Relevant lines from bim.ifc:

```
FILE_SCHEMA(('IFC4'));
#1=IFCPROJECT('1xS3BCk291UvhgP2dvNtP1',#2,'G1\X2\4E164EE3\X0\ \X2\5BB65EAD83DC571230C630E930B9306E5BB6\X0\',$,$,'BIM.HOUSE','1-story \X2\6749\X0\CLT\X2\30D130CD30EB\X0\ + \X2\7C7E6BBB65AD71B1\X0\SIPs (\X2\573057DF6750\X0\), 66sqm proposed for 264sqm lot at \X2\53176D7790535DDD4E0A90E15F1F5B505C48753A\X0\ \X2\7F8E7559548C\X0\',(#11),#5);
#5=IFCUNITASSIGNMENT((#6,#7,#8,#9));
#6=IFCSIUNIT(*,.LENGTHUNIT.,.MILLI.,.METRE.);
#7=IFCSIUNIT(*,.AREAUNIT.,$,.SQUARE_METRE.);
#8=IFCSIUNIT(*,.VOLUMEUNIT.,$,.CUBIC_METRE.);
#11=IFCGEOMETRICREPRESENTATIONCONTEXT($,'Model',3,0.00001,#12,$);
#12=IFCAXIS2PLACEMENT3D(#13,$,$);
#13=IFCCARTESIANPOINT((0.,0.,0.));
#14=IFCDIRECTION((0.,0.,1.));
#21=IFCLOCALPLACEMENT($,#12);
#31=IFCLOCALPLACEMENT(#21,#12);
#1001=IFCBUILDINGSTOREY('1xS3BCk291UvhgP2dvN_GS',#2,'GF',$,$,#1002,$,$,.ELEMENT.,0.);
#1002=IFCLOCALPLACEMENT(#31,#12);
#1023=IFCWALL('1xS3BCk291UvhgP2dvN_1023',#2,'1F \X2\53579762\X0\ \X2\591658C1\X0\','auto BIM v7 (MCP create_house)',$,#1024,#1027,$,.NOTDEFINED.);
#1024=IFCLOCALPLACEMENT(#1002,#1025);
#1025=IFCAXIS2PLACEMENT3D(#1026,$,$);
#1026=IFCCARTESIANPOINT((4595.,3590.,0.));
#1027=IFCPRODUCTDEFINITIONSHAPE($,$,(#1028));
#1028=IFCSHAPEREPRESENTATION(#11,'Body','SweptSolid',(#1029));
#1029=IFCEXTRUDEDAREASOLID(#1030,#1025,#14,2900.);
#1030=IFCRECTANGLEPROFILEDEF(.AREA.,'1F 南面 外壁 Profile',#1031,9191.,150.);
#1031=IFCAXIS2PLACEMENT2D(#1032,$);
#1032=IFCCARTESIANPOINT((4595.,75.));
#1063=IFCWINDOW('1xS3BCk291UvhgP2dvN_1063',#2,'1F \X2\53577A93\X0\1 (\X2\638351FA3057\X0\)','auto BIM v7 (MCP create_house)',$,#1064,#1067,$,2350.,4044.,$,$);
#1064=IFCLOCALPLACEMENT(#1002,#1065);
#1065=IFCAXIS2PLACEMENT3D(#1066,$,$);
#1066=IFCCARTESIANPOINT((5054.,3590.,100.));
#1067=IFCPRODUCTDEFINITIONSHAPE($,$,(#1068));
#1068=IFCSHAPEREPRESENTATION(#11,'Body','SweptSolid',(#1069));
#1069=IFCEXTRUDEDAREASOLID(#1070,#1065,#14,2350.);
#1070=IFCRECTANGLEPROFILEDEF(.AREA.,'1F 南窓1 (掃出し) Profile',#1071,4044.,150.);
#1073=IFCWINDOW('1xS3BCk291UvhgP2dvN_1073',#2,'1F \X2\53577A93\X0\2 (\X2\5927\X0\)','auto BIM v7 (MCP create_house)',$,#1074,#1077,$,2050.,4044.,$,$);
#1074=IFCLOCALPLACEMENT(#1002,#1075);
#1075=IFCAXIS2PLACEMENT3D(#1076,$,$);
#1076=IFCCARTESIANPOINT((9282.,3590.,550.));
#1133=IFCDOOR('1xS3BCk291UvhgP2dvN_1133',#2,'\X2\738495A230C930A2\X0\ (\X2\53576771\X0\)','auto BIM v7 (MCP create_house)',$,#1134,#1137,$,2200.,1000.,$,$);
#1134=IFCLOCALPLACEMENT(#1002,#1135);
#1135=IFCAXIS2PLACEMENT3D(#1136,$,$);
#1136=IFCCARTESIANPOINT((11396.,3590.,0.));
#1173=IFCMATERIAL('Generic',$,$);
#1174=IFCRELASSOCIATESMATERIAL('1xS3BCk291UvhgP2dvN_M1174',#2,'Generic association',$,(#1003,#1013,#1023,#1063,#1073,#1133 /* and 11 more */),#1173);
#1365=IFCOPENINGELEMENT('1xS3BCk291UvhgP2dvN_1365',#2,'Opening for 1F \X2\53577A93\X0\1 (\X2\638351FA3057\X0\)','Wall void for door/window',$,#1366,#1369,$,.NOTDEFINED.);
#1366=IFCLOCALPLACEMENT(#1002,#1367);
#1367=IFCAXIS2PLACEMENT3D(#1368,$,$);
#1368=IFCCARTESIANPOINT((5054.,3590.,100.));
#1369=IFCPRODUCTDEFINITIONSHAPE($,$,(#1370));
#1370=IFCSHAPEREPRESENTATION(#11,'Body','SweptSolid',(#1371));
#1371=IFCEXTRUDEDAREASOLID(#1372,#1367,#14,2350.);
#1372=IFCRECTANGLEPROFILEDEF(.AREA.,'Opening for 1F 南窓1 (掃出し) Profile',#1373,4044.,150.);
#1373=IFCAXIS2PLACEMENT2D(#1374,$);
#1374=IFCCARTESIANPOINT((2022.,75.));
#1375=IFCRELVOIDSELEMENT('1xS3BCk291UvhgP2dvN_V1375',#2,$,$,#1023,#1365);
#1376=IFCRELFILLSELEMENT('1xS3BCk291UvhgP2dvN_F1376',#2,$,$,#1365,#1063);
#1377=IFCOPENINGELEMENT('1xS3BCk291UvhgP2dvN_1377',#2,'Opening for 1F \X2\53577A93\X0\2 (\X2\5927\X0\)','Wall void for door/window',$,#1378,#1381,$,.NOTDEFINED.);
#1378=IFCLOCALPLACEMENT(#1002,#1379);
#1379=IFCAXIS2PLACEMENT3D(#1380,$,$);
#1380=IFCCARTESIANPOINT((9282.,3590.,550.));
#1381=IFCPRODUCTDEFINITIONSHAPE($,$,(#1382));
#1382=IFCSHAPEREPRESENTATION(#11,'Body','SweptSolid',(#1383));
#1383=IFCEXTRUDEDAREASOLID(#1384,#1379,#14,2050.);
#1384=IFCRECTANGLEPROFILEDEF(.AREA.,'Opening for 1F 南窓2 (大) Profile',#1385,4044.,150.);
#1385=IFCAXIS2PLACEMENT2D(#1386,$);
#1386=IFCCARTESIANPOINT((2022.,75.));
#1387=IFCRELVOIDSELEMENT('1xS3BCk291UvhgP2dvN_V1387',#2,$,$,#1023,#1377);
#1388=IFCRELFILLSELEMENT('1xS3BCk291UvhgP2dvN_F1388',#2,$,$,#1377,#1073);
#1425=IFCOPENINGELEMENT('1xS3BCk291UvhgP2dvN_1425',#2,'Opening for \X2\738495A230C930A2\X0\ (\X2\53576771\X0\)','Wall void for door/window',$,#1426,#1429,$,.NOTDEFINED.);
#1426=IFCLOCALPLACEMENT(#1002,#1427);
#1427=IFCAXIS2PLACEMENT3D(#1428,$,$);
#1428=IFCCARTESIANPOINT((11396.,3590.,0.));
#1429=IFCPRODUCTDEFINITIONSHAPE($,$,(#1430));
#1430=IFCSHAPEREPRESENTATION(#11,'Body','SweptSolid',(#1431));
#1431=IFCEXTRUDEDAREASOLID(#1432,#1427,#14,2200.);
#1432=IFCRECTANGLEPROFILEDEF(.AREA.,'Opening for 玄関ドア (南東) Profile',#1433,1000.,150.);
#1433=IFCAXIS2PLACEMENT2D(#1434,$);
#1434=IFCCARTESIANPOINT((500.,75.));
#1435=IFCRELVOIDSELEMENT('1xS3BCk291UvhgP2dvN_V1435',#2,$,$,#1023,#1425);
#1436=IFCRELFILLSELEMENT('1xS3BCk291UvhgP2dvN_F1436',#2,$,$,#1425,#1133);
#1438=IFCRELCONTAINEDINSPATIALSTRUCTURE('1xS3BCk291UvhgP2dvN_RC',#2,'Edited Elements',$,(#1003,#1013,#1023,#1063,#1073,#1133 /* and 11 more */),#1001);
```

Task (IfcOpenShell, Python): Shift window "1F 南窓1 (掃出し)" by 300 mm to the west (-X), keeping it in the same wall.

```python
import ifcopenshell
import ifcopenshell.api.geometry
import ifcopenshell.util.placement
import ifcopenshell.util.unit

model = ifcopenshell.open("bim.ifc")
unit_scale = ifcopenshell.util.unit.calculate_unit_scale(model)

window = model.by_guid("1xS3BCk291UvhgP2dvN_1063")
opening = window.FillsVoids[0].RelatingOpeningElement
wall = opening.VoidsElements[0].RelatingBuildingElement

wall_matrix = ifcopenshell.util.placement.get_local_placement(wall.ObjectPlacement)
shift = wall_matrix[:3, 0] * -0.3 / unit_scale
before = ifcopenshell.util.placement.get_local_placement(window.ObjectPlacement)[:3, 3].copy()

# The window is not placed relative to its opening, so move both.
for product in (opening, window):
    matrix = ifcopenshell.util.placement.get_local_placement(product.ObjectPlacement)
    matrix[:3, 3] += shift
    ifcopenshell.api.geometry.edit_object_placement(model, product=product, matrix=matrix, is_si=False)

after = ifcopenshell.util.placement.get_local_placement(window.ObjectPlacement)[:3, 3]
print("window moved by", (after - before).round(3) + 0.0)

model.write("bim_rev.ifc")
```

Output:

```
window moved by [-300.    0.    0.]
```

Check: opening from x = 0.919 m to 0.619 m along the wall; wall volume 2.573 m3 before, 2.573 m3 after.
